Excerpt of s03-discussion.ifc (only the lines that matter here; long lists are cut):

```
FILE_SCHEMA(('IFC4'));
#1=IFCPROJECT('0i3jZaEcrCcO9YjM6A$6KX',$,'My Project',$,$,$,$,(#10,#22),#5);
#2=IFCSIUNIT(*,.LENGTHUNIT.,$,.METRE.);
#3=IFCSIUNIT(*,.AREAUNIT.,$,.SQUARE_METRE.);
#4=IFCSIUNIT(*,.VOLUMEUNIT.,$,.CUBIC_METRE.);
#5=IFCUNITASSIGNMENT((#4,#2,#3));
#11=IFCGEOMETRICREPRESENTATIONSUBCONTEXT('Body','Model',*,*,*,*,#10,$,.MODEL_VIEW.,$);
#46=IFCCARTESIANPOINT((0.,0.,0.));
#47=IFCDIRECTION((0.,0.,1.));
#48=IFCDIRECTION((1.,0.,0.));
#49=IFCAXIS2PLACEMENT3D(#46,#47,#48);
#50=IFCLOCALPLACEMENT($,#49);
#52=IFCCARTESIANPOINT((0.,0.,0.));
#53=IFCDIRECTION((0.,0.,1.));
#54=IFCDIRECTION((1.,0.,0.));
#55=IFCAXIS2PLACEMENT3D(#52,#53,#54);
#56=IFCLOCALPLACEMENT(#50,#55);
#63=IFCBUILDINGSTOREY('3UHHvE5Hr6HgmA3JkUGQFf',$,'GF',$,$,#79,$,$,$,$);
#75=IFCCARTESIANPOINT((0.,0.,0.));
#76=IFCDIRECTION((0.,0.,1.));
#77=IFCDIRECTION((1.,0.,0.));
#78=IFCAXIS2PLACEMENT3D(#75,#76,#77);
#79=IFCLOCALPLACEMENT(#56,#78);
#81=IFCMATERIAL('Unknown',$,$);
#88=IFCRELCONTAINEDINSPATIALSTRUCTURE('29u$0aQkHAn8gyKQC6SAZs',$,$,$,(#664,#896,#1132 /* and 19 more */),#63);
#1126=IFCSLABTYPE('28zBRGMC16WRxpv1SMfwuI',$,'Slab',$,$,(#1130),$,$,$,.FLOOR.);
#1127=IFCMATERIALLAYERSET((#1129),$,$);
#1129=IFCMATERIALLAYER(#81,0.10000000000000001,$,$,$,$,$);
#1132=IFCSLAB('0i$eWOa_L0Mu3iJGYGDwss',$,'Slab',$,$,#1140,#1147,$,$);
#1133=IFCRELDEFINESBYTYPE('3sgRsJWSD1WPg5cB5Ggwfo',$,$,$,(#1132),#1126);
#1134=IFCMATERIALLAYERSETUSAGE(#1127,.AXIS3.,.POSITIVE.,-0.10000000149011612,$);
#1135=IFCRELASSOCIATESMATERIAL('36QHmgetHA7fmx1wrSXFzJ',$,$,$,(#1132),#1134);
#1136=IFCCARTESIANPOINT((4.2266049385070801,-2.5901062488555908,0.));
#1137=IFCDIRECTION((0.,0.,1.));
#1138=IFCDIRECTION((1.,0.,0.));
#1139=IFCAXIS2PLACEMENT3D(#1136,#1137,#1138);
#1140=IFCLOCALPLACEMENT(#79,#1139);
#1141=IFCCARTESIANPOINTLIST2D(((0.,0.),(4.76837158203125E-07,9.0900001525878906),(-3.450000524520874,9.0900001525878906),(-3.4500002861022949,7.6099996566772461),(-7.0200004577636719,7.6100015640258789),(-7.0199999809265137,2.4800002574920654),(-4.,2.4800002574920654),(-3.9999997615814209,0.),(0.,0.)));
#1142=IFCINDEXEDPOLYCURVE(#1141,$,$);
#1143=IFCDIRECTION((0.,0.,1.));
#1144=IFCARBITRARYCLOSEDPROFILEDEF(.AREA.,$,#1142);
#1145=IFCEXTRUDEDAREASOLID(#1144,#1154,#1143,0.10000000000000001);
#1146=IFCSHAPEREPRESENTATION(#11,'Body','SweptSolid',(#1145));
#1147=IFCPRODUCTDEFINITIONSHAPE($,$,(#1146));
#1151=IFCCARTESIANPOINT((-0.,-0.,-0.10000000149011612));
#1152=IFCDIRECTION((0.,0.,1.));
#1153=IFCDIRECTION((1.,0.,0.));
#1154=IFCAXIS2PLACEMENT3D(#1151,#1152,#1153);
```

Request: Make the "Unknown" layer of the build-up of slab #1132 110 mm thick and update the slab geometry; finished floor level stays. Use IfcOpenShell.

```python
import ifcopenshell
import ifcopenshell.util.element
import ifcopenshell.util.representation
import ifcopenshell.util.unit

model = ifcopenshell.open("s03-discussion.ifc")
unit_scale = ifcopenshell.util.unit.calculate_unit_scale(model)

layer_set = model.by_id(1127)
layer = next(l for l in layer_set.MaterialLayers if l.Material and l.Material.Name == "Unknown")
change = 0.11 / unit_scale - layer.LayerThickness
layer.LayerThickness += change

# Geometry does not follow the layer set by itself.
slabs = [e for e in ifcopenshell.util.element.get_elements_by_material(model, layer_set) if e.is_a("IfcSlab")]
for slab in sorted(slabs, key=lambda e: e.id()):
    body = ifcopenshell.util.representation.get_representation(slab, "Model", "Body")
    solid = body.Items[0]
    old_depth = solid.Depth
    solid.Depth += change
    # Extruded upwards: lower the start of the extrusion so the top stays.
    x, y, z = solid.Position.Location.Coordinates
    solid.Position.Location = model.createIfcCartesianPoint((x, y, z - change))
    print(slab.id(), f"{old_depth:g} -> {solid.Depth:g}")

# The layers are counted up from the underside, which has moved.
for usage in {ifcopenshell.util.element.get_material(slab) for slab in slabs}:
    usage.OffsetFromReferenceLine -= change

model.write("s03-discussion_updated.ifc")
```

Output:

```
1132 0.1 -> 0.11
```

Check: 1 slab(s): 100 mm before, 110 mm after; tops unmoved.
